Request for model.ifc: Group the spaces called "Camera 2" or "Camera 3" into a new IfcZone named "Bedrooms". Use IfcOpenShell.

First a look at what the model holds.

```python
import ifcopenshell

model = ifcopenshell.open("model.ifc")
print(model.schema)
seen = {}
for space in model.by_type("IfcSpace"):
    seen[space.LongName] = seen.get(space.LongName, 0) + 1
for name, count in sorted(seen.items(), key=str):
    print(count, "x", name)
print("zones:", [z.Name for z in model.by_type("IfcZone")][:20])
```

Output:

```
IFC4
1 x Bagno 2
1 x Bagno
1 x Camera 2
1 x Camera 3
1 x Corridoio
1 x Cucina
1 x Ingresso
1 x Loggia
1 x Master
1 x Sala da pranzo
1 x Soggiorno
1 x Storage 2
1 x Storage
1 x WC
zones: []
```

```python
import ifcopenshell
import ifcopenshell.api.group
import ifcopenshell.api.root

model = ifcopenshell.open("model.ifc")

names = {"Camera 2", "Camera 3"}
spaces = [s for s in model.by_type("IfcSpace") if s.LongName in names]

zone = ifcopenshell.api.root.create_entity(model, ifc_class="IfcZone", name="Bedrooms")
ifcopenshell.api.group.assign_group(model, products=spaces, group=zone)
print(len(spaces), "spaces in", zone.Name)

model.write("model_rev.ifc")
```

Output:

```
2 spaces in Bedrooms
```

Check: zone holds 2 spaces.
